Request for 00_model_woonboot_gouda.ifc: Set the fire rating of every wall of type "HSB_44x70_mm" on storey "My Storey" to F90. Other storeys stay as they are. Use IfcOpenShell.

First a look at what the model holds.

```python
import ifcopenshell
import ifcopenshell.util.element

model = ifcopenshell.open("00_model_woonboot_gouda.ifc")
print(model.schema)
storey = next(s for s in model.by_type("IfcBuildingStorey") if s.Name == "My Storey")
walls = [e for e in ifcopenshell.util.element.get_decomposition(storey) if e.is_a("IfcWall")]
seen = {}
for e in walls:
    element_type = ifcopenshell.util.element.get_type(e)
    key = (element_type.Name if element_type != e and element_type else None, ifcopenshell.util.element.get_pset(e, "Pset_WallCommon", "FireRating"))
    seen[key] = seen.get(key, 0) + 1
for (name, value), count in sorted(seen.items(), key=str):
    print(count, "x", name, "|", value)
```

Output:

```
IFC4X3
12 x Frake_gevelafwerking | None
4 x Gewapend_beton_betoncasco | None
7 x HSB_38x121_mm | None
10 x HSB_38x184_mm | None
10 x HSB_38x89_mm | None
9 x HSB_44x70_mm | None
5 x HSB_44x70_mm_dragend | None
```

```python
import ifcopenshell
import ifcopenshell.api.pset
import ifcopenshell.util.element

model = ifcopenshell.open("00_model_woonboot_gouda.ifc")

storey = next(s for s in model.by_type("IfcBuildingStorey") if s.Name == "My Storey")
walls = [e for e in ifcopenshell.util.element.get_decomposition(storey) if e.is_a("IfcWall")]

count = 0
for e in walls:
    element_type = ifcopenshell.util.element.get_type(e)
    if element_type in (None, e) or element_type.Name != "HSB_44x70_mm":
        continue
    # add_pset returns the element's existing set when there is one.
    pset = ifcopenshell.api.pset.add_pset(model, product=e, name="Pset_WallCommon")
    ifcopenshell.api.pset.edit_pset(model, pset=pset, properties={"FireRating": "F90"})
    count += 1

print(count, "walls updated")

model.write("00_model_woonboot_gouda_rev.ifc")
```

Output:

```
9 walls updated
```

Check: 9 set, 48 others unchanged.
